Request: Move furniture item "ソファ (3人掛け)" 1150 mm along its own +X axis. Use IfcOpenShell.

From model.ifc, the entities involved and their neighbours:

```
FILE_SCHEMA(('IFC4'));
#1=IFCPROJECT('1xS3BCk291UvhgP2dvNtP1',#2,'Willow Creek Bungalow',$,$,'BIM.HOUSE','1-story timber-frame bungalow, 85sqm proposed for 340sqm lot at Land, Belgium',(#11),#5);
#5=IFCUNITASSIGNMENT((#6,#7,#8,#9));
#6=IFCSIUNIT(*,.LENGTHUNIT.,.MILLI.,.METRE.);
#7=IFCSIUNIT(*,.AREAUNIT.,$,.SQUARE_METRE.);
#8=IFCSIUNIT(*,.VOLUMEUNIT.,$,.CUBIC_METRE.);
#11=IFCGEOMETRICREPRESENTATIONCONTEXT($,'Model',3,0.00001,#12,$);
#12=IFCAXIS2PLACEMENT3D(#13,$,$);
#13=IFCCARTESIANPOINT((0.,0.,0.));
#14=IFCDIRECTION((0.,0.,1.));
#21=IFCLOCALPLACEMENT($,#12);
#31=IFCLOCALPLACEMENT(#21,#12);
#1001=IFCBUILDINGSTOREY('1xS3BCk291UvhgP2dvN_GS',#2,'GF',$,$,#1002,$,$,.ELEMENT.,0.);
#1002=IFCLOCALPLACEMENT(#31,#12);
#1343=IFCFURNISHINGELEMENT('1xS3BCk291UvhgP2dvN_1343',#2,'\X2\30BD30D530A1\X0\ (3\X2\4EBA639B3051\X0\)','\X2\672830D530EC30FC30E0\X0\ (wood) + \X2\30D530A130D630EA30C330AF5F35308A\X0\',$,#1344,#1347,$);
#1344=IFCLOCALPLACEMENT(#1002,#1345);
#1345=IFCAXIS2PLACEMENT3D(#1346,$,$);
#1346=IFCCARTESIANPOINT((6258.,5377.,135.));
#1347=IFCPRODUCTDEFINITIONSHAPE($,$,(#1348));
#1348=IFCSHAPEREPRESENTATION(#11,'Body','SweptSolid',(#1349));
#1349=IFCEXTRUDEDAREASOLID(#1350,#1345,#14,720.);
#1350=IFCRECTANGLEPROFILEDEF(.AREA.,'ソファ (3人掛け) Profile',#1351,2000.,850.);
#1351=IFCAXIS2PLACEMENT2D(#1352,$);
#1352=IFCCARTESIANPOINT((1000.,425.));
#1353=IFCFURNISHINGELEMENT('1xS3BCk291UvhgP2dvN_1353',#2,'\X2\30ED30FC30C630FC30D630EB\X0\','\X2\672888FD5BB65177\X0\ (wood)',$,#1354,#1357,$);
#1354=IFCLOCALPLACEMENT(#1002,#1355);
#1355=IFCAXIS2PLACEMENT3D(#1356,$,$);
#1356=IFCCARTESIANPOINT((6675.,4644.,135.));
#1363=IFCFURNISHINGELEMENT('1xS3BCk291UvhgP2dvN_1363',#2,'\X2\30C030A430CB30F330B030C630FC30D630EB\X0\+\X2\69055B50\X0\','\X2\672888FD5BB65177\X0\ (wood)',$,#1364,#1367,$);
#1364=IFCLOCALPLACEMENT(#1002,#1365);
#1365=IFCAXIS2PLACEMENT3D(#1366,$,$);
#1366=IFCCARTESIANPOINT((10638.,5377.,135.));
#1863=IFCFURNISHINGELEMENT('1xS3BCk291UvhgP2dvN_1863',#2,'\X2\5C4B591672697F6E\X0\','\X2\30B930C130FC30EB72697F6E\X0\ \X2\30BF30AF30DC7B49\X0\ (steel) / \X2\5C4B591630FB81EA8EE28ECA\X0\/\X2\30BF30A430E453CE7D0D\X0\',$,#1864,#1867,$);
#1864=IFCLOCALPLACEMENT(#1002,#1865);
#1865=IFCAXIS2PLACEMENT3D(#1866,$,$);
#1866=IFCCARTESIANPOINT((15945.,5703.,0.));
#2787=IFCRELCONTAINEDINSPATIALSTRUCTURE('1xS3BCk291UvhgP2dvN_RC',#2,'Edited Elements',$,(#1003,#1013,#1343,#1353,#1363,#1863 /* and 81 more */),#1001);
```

```python
import ifcopenshell
import ifcopenshell.api.geometry
import ifcopenshell.util.placement

model = ifcopenshell.open("model.ifc")

item = model.by_guid("1xS3BCk291UvhgP2dvN_1343")
matrix = ifcopenshell.util.placement.get_local_placement(item.ObjectPlacement)
matrix[:3, 3] += matrix[:3, 0] * 1150.0
ifcopenshell.api.geometry.edit_object_placement(model, product=item, matrix=matrix, is_si=False)

print(ifcopenshell.util.placement.get_local_placement(item.ObjectPlacement).round(3) + 0.0)

model.write("model_updated.ifc")
```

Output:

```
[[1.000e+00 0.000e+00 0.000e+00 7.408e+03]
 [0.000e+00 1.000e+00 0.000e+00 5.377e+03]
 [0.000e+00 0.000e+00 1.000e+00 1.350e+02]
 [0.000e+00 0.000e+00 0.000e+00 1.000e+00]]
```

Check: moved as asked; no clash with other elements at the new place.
